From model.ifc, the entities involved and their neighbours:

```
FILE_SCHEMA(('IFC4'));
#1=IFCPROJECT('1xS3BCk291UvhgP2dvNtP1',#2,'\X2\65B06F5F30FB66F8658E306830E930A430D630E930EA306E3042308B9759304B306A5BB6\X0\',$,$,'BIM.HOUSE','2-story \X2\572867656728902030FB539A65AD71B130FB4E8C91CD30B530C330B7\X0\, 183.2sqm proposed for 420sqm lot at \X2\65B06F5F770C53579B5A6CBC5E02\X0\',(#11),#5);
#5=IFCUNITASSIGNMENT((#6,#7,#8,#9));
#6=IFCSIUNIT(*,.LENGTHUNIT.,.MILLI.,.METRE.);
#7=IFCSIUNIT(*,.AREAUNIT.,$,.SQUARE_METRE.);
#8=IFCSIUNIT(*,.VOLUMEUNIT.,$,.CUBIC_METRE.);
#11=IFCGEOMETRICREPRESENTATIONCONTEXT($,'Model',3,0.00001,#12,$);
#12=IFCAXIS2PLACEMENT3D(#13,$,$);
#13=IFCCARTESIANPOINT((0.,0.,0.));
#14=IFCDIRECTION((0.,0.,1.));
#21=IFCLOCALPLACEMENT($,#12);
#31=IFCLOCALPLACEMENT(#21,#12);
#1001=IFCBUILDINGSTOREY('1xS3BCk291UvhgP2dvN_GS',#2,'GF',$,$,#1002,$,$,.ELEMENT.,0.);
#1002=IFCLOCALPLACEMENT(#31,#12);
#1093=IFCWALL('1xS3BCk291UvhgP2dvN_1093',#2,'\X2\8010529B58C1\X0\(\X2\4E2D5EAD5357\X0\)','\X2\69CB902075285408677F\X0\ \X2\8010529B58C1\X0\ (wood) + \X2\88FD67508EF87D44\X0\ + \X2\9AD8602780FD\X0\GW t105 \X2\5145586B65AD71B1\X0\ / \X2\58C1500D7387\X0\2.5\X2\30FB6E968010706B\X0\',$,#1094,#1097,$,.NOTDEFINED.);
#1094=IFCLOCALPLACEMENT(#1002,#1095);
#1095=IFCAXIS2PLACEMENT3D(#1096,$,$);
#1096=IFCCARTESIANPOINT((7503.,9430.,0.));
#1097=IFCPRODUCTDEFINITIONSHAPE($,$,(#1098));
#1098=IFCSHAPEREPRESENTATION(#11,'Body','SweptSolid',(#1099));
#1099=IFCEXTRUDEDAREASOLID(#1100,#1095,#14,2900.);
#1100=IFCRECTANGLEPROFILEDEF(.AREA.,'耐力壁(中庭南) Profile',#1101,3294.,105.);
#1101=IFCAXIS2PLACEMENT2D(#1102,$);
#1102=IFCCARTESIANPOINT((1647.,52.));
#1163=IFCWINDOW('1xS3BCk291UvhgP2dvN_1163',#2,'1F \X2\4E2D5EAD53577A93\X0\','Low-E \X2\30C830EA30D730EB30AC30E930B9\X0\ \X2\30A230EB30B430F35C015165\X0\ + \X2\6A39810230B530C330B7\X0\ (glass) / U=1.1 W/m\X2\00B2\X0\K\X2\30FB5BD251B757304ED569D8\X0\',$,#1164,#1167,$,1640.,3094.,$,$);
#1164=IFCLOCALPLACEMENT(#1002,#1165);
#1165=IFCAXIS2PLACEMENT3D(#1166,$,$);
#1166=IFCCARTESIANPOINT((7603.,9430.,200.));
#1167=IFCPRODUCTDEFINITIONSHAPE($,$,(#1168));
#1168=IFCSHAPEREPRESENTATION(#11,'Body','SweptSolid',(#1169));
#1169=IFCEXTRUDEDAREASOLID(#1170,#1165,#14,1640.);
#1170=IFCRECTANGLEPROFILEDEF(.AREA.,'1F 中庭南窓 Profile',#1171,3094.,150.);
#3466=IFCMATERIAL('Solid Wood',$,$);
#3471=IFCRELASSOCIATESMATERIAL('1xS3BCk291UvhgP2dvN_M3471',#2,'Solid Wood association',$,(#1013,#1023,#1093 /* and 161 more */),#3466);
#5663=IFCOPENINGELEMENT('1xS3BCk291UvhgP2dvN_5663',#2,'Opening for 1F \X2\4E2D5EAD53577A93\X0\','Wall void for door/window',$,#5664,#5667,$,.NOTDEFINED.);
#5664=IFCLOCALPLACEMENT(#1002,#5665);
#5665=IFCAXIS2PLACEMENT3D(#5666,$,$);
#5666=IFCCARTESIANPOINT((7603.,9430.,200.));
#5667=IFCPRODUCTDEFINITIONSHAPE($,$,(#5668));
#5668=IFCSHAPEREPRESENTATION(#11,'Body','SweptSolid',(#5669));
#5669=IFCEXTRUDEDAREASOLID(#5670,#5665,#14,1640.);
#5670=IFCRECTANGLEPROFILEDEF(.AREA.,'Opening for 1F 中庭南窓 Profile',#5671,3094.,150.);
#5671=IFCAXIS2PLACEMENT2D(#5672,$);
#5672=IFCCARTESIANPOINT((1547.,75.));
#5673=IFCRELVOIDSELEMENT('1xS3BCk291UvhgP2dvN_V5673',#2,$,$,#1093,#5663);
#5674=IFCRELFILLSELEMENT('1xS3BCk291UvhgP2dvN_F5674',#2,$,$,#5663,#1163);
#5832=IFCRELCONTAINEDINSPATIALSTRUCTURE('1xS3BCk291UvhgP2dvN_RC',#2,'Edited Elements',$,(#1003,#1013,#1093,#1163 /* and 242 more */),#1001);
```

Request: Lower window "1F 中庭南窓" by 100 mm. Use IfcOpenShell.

```python
import numpy as np
import ifcopenshell
import ifcopenshell.api.geometry
import ifcopenshell.util.placement
import ifcopenshell.util.unit

model = ifcopenshell.open("model.ifc")
unit_scale = ifcopenshell.util.unit.calculate_unit_scale(model)

window = model.by_id(1163)
opening = window.FillsVoids[0].RelatingOpeningElement
dz = -100.0

shift = np.array([0.0, 0.0, dz])
# The window is not placed relative to its opening, so move both.
for product in (opening, window):
    matrix = ifcopenshell.util.placement.get_local_placement(product.ObjectPlacement)
    matrix[:3, 3] += shift
    ifcopenshell.api.geometry.edit_object_placement(model, product=product, matrix=matrix, is_si=False)

print(f"moved by {dz * unit_scale:+.3f} m")

model.write("model-out.ifc")
```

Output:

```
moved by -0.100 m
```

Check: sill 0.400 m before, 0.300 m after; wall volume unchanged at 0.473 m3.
